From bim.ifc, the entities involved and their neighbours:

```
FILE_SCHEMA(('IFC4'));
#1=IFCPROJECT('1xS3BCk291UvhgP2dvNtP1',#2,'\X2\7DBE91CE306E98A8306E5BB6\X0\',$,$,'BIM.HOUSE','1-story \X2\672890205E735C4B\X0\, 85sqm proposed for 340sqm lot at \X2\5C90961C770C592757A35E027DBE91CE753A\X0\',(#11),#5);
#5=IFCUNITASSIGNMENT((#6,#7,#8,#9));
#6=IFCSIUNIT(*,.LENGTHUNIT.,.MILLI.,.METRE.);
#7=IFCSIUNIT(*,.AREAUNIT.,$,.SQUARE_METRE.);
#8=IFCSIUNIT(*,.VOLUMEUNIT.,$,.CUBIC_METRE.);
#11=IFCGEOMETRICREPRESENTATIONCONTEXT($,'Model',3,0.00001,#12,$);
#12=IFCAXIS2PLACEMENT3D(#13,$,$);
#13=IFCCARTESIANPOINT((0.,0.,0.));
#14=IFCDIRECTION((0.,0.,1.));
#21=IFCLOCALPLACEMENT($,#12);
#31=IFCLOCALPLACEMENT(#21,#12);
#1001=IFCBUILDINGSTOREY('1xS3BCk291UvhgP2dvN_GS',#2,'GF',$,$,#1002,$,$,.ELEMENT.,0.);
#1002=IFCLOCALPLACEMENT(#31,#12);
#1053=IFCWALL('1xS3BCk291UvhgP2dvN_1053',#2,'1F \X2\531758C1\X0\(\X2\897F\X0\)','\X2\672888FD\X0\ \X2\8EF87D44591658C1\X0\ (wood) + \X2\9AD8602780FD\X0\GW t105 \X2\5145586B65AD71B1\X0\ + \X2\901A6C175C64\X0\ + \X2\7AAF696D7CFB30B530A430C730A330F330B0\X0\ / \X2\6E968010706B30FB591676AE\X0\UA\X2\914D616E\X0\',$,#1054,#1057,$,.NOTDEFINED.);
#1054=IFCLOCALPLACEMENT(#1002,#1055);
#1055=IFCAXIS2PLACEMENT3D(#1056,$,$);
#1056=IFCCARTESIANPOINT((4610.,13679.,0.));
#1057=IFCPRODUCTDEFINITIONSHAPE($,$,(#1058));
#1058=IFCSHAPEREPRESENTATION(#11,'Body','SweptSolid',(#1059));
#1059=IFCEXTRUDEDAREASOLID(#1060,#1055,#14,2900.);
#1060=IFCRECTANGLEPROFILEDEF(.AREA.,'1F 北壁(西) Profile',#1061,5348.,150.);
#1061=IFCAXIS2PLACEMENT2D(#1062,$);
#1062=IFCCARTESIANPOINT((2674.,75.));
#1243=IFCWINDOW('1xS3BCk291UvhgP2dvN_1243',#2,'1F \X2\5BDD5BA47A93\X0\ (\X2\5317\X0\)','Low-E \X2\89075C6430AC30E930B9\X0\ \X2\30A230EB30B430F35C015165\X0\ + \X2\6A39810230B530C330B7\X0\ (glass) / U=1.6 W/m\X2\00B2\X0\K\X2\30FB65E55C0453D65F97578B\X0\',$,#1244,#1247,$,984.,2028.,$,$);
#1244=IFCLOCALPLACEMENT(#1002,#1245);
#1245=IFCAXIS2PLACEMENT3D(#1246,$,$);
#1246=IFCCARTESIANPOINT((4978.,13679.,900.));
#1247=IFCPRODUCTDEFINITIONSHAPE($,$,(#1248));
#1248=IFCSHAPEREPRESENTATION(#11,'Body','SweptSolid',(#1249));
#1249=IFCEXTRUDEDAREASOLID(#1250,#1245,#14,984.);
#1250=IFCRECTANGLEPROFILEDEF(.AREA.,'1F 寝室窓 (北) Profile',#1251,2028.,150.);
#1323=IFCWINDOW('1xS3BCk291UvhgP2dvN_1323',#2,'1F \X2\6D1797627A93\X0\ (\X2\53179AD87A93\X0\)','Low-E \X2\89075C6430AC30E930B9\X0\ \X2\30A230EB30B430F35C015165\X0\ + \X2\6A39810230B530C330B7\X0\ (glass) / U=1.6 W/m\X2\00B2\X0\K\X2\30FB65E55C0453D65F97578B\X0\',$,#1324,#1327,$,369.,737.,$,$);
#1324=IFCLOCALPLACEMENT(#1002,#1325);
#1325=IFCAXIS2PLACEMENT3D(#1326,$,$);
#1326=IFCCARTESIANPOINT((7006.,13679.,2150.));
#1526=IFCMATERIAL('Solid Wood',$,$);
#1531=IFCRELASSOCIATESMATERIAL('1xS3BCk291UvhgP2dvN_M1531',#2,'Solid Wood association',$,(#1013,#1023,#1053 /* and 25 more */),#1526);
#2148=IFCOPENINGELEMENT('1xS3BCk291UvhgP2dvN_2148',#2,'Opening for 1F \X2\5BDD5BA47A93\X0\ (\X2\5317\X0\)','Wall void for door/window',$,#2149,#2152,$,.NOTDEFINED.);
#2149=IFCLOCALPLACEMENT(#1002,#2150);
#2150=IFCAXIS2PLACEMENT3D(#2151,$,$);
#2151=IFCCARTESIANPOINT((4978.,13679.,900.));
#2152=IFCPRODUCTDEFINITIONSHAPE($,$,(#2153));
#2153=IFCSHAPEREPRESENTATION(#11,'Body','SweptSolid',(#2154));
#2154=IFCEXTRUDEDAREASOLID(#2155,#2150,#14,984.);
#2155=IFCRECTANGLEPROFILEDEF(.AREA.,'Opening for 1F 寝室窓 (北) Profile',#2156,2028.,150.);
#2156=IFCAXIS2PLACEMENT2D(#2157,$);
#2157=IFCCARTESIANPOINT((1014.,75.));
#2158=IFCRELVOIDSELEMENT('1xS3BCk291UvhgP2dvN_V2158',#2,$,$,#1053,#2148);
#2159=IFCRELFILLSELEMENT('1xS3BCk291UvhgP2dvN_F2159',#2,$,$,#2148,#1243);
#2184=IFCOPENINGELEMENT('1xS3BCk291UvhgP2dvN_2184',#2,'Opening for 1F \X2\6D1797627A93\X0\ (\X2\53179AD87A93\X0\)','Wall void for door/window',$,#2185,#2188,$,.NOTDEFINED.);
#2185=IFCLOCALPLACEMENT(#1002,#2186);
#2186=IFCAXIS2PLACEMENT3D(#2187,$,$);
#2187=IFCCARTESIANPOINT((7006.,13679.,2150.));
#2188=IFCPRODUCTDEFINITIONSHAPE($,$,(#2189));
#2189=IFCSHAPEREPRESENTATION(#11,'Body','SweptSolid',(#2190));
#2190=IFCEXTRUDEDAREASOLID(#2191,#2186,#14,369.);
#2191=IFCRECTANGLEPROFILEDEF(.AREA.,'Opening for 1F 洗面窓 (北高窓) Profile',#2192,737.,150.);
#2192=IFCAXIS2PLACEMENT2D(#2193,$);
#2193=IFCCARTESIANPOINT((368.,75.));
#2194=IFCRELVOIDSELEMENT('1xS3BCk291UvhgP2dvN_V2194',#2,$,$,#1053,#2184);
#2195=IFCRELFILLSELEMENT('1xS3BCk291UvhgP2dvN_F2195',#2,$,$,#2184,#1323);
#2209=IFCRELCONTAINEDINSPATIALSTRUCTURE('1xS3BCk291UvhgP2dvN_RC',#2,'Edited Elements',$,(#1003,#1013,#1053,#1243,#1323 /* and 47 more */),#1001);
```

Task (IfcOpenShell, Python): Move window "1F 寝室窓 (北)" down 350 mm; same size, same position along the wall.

```python
import numpy as np
import ifcopenshell
import ifcopenshell.api.geometry
import ifcopenshell.util.placement
import ifcopenshell.util.unit

model = ifcopenshell.open("bim.ifc")
unit_scale = ifcopenshell.util.unit.calculate_unit_scale(model)

window = model.by_guid("1xS3BCk291UvhgP2dvN_1243")
opening = window.FillsVoids[0].RelatingOpeningElement
dz = -0.35 / unit_scale

shift = np.array([0.0, 0.0, dz])
# The window is not placed relative to its opening, so move both.
for product in (opening, window):
    matrix = ifcopenshell.util.placement.get_local_placement(product.ObjectPlacement)
    matrix[:3, 3] += shift
    ifcopenshell.api.geometry.edit_object_placement(model, product=product, matrix=matrix, is_si=False)

print(f"moved by {dz * unit_scale:+.3f} m")

model.write("bim_v2.ifc")
```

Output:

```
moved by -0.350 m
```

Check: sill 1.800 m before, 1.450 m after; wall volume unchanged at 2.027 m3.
